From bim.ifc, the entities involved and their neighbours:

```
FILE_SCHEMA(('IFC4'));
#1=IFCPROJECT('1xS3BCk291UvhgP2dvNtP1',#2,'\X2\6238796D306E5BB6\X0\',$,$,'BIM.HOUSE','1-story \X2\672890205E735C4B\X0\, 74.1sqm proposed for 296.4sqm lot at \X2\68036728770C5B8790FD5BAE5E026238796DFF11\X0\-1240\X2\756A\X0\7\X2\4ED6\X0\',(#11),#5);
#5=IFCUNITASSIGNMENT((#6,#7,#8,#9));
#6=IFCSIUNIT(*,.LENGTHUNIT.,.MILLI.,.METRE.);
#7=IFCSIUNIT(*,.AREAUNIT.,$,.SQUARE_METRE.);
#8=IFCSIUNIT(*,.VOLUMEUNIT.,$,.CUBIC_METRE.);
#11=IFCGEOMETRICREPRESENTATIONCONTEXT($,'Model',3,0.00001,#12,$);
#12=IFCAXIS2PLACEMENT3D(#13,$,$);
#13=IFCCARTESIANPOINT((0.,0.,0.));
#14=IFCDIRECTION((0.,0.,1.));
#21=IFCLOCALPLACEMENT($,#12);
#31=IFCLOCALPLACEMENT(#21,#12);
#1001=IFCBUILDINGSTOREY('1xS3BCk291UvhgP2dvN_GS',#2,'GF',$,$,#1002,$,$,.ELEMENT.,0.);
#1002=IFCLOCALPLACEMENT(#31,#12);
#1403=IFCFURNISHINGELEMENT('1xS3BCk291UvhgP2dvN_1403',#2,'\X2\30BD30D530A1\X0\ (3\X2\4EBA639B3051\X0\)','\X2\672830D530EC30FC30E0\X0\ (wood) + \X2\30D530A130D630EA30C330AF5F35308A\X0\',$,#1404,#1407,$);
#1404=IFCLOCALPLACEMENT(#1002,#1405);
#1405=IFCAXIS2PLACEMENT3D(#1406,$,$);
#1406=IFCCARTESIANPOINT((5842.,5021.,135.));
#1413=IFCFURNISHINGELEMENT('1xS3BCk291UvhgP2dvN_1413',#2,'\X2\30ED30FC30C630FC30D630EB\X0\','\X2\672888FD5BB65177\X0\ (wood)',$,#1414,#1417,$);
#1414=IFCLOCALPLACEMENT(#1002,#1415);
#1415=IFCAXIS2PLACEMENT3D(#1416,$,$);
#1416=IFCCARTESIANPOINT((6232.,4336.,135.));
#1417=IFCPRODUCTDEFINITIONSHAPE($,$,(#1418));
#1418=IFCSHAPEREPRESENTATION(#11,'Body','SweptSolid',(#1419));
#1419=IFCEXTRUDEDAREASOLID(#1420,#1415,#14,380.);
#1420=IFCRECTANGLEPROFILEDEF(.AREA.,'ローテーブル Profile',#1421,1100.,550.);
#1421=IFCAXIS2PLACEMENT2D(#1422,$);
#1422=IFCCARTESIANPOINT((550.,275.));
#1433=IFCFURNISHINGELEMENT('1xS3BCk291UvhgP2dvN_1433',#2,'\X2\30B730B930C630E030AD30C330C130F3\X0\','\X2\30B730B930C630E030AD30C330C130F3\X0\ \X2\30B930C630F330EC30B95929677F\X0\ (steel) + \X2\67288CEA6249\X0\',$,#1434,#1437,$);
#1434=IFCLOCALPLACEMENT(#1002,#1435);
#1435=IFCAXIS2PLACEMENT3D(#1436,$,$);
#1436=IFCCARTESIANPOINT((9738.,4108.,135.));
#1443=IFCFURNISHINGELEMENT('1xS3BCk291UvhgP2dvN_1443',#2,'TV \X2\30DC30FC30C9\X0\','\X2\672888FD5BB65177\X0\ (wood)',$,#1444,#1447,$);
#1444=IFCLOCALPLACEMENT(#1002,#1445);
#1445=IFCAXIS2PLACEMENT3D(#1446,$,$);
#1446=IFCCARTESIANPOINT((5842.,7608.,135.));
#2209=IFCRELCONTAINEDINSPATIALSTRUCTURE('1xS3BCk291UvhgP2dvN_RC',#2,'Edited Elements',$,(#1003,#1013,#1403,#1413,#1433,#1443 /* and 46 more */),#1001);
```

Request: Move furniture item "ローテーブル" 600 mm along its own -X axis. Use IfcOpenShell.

```python
import ifcopenshell
import ifcopenshell.api.geometry
import ifcopenshell.util.placement
import ifcopenshell.util.unit

model = ifcopenshell.open("bim.ifc")
unit_scale = ifcopenshell.util.unit.calculate_unit_scale(model)

item = model.by_guid("1xS3BCk291UvhgP2dvN_1413")
matrix = ifcopenshell.util.placement.get_local_placement(item.ObjectPlacement)
matrix[:3, 3] -= matrix[:3, 0] * 0.6 / unit_scale
ifcopenshell.api.geometry.edit_object_placement(model, product=item, matrix=matrix, is_si=False)

print(ifcopenshell.util.placement.get_local_placement(item.ObjectPlacement).round(3) + 0.0)

model.write("bim_v2.ifc")
```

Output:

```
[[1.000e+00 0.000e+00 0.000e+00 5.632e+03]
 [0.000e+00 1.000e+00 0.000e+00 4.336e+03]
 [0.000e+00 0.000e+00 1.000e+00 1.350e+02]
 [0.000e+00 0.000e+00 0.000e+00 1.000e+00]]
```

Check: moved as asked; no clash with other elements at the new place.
